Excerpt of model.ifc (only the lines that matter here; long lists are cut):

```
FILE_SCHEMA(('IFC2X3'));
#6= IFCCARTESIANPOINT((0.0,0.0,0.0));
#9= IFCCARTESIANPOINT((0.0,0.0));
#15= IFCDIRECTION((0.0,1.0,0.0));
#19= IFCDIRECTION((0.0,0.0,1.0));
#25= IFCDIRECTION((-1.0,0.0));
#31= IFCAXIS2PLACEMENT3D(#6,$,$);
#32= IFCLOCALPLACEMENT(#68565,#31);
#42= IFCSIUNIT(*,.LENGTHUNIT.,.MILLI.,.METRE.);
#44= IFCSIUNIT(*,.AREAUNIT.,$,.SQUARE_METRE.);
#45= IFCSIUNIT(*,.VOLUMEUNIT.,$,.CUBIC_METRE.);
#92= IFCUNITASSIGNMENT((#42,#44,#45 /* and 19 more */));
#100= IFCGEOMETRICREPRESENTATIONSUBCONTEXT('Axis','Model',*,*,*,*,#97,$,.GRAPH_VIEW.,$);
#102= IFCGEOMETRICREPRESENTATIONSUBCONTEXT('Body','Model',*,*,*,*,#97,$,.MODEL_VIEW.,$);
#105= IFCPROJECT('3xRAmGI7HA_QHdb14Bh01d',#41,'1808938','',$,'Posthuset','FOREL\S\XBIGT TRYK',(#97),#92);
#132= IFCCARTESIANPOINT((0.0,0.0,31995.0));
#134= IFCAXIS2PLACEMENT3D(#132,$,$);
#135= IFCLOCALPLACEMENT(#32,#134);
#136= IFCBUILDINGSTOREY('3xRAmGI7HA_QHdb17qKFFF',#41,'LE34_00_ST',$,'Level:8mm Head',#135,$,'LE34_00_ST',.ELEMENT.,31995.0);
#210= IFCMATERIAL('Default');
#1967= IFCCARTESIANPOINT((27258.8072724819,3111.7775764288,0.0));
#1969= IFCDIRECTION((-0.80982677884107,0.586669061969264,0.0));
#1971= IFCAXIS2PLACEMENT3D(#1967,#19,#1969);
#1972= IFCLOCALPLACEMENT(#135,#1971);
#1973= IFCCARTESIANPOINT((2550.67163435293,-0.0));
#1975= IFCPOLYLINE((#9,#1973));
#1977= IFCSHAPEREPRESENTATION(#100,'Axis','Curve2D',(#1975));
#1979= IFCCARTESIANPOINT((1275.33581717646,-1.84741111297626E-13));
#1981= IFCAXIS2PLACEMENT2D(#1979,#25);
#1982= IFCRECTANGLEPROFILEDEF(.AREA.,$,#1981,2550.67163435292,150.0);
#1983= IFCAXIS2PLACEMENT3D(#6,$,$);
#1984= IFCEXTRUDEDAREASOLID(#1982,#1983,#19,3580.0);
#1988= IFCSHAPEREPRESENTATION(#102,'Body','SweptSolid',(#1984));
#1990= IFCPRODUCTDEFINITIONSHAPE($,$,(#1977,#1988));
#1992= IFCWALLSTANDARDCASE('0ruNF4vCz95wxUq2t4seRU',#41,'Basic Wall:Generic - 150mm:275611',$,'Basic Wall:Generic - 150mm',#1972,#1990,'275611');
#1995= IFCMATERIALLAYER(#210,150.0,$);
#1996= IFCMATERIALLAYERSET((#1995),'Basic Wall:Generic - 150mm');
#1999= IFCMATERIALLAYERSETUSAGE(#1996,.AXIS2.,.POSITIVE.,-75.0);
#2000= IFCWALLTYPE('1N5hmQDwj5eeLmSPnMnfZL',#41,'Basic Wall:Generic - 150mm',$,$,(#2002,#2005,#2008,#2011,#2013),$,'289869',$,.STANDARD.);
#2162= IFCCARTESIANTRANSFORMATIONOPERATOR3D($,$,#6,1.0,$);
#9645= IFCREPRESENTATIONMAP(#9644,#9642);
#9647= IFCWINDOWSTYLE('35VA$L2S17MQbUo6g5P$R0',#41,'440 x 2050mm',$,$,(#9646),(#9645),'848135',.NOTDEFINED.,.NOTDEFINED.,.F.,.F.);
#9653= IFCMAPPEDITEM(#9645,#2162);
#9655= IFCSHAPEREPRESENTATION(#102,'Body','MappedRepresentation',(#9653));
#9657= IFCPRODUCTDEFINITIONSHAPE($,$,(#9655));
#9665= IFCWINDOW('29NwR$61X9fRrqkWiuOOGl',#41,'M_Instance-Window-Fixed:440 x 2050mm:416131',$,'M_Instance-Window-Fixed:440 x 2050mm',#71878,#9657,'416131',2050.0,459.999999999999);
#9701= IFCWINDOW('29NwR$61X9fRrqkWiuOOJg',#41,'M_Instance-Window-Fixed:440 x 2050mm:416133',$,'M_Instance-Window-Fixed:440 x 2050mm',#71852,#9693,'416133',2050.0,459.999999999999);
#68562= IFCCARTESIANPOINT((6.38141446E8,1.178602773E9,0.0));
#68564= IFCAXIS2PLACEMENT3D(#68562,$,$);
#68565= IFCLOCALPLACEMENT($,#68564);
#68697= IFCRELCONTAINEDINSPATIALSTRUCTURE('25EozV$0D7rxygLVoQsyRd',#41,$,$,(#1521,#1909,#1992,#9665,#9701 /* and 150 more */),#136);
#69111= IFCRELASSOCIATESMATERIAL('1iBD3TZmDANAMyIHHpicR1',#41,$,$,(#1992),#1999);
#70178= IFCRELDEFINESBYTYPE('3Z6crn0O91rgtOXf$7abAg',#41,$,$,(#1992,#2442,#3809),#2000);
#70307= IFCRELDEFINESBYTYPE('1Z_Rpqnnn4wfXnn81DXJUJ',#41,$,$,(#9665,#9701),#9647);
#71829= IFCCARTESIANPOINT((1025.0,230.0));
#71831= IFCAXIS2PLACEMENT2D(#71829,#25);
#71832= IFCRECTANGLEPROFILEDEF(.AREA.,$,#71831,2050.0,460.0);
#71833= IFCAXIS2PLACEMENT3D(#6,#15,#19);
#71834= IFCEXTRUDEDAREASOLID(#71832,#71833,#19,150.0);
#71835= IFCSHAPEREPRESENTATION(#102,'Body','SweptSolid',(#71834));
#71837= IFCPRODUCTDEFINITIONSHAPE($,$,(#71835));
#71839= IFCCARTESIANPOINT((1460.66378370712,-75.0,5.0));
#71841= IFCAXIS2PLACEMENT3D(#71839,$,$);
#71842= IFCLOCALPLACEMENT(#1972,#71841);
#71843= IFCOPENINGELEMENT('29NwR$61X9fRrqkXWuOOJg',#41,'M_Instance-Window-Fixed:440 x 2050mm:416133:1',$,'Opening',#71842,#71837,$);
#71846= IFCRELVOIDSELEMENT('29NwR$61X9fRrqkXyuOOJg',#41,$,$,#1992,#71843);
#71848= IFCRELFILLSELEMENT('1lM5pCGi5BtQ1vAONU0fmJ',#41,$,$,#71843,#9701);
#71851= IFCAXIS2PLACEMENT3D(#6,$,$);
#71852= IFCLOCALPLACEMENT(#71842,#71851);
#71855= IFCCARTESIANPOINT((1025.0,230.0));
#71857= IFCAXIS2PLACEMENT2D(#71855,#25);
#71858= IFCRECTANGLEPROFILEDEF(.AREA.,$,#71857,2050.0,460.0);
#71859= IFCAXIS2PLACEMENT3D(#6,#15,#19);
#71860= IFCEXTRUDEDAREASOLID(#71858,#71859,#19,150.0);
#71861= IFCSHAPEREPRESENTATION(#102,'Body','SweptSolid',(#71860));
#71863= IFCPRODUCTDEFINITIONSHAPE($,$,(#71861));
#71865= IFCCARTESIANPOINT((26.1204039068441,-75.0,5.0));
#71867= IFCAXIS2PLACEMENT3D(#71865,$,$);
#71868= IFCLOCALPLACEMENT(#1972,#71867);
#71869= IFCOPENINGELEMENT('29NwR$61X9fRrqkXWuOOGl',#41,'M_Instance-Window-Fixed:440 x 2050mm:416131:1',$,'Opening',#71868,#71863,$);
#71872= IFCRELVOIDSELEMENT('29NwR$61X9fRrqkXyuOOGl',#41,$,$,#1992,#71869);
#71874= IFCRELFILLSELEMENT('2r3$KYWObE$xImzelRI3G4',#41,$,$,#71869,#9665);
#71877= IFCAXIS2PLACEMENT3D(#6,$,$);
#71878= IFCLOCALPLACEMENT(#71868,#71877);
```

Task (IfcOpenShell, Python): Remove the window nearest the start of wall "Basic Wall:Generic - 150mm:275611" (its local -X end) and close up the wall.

```python
import ifcopenshell
import ifcopenshell.api.feature
import ifcopenshell.api.root
import ifcopenshell.geom
import ifcopenshell.util.shape

model = ifcopenshell.open("model.ifc")
settings = ifcopenshell.geom.settings()


def volume(element):
    """Net volume in cubic metres, openings subtracted."""
    shape = ifcopenshell.geom.create_shape(settings, element)
    return ifcopenshell.util.shape.get_volume(shape.geometry)


window = model.by_id(9665)
opening = window.FillsVoids[0].RelatingOpeningElement
wall = opening.VoidsElements[0].RelatingBuildingElement
before = volume(wall)

ifcopenshell.api.root.remove_product(model, product=window)
ifcopenshell.api.feature.remove_feature(model, feature=opening)

after = volume(wall)

print(f"wall volume {before:.3f} -> {after:.3f} m3")

model.write("model_rev.ifc")
```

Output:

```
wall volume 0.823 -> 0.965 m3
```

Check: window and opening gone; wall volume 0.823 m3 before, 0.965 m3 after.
